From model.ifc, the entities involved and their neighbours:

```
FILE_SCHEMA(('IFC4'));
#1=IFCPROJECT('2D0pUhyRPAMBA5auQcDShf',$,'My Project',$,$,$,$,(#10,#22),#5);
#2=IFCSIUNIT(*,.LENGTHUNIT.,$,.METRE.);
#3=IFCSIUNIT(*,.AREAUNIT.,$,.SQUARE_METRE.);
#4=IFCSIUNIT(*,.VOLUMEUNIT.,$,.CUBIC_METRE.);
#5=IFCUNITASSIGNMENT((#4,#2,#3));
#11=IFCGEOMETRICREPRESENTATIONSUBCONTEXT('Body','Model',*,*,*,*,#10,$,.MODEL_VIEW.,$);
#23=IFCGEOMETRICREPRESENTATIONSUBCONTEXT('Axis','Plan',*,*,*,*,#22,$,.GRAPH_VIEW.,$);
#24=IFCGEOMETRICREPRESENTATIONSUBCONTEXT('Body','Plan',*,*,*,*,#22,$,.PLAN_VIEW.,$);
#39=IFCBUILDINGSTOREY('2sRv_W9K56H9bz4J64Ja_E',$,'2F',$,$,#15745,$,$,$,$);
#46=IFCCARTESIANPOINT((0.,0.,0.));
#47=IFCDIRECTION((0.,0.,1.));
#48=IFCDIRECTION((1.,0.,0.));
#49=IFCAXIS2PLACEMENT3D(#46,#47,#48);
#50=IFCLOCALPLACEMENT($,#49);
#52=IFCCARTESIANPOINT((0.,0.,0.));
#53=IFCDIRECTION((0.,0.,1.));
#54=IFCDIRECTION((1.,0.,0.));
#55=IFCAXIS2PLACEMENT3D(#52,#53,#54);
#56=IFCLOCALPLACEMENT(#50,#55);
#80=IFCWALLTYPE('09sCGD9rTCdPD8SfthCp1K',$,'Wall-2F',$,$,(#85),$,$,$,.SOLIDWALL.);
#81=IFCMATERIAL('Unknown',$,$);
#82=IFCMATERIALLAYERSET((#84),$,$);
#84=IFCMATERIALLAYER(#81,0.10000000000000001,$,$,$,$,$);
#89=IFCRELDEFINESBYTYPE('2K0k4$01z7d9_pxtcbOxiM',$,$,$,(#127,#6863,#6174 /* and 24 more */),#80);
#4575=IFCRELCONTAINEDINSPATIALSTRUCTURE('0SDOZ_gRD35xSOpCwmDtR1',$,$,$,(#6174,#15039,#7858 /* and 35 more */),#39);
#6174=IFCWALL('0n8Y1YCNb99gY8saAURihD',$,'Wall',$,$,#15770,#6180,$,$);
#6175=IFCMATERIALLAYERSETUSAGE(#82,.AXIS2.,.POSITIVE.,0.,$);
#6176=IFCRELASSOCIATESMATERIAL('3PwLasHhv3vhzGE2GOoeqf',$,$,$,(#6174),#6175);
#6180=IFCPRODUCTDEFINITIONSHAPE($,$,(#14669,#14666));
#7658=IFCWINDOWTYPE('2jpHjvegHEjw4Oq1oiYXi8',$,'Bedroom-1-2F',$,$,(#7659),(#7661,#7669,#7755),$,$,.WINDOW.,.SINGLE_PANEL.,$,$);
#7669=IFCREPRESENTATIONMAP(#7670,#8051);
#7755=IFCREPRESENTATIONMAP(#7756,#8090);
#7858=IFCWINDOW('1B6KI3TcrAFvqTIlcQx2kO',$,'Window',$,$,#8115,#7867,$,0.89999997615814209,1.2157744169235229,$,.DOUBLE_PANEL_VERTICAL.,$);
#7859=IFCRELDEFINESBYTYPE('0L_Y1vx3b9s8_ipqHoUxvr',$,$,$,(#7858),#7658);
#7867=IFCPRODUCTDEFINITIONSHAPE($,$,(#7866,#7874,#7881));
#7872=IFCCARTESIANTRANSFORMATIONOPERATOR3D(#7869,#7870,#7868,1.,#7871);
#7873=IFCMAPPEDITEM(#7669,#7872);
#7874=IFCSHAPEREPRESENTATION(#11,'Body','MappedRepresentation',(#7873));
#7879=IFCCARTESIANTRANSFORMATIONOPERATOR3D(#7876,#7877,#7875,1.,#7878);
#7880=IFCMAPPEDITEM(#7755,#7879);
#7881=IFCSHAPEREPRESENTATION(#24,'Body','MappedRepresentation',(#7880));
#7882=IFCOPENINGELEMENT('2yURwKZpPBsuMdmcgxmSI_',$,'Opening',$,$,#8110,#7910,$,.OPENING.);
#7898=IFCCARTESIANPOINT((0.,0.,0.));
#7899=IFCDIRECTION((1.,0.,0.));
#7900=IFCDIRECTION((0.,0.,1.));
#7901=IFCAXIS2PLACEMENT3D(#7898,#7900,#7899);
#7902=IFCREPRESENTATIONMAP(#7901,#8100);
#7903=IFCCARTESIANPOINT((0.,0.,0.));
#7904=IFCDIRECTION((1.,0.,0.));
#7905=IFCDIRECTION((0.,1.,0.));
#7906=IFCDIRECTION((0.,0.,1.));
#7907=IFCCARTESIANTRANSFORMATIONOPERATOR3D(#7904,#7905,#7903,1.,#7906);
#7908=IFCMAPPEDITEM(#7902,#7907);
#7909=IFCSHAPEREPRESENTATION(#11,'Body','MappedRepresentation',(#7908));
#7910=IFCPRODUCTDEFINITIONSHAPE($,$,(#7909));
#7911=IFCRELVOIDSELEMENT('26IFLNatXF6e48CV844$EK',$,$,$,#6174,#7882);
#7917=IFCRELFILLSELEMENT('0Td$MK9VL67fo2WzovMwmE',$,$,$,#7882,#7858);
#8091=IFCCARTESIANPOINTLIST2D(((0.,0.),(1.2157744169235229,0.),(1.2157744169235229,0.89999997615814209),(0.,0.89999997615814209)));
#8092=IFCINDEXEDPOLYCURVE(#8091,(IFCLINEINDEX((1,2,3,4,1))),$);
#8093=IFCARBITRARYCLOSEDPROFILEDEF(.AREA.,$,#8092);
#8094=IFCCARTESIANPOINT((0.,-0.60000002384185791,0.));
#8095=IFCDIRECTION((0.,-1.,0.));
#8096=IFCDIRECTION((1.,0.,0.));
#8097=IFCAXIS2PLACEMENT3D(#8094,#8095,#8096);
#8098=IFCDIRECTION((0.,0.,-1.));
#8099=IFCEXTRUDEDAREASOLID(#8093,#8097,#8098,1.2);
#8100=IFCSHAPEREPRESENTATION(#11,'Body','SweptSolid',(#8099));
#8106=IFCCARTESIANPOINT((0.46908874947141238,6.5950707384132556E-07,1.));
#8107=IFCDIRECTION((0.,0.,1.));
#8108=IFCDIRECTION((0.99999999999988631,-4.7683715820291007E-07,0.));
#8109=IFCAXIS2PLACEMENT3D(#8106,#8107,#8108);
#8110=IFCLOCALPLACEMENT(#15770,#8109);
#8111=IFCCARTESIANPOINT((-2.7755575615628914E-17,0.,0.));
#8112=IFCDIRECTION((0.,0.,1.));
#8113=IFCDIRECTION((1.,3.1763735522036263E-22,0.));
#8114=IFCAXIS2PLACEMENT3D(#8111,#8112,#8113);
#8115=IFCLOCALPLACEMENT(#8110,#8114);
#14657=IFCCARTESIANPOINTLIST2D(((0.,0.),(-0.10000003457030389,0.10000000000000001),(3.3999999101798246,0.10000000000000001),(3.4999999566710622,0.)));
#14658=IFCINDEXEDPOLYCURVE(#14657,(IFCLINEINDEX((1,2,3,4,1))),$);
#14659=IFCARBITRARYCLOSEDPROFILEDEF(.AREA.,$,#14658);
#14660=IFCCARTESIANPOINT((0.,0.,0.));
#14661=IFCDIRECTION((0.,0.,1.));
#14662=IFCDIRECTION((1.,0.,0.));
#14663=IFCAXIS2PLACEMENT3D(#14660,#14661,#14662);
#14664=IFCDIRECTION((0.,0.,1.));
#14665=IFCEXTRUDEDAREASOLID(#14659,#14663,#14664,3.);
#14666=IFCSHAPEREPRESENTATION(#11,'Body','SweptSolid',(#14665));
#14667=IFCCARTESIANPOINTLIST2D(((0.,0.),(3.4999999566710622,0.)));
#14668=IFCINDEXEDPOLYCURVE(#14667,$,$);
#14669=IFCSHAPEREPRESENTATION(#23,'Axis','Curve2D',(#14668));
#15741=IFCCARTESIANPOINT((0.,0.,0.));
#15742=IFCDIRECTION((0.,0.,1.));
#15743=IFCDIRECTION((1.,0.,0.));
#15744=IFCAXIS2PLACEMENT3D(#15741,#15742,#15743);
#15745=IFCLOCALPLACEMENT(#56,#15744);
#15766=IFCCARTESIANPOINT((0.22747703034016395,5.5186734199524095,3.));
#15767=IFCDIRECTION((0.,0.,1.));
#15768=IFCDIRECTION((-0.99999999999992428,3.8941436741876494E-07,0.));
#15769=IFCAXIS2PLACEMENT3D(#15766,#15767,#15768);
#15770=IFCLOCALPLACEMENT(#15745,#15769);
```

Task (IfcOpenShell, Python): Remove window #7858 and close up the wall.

```python
import ifcopenshell
import ifcopenshell.api.feature
import ifcopenshell.api.root
import ifcopenshell.geom
import ifcopenshell.util.shape

model = ifcopenshell.open("model.ifc")
settings = ifcopenshell.geom.settings()


def volume(element):
    """Net volume in cubic metres, openings subtracted."""
    shape = ifcopenshell.geom.create_shape(settings, element)
    return ifcopenshell.util.shape.get_volume(shape.geometry)


window = model.by_id(7858)
opening = window.FillsVoids[0].RelatingOpeningElement
wall = opening.VoidsElements[0].RelatingBuildingElement
before = volume(wall)

ifcopenshell.api.root.remove_product(model, product=window)
ifcopenshell.api.feature.remove_feature(model, feature=opening)

after = volume(wall)

print(f"wall volume {before:.3f} -> {after:.3f} m3")

model.write("model_v2.ifc")
```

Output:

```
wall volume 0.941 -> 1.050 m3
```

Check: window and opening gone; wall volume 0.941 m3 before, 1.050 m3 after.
